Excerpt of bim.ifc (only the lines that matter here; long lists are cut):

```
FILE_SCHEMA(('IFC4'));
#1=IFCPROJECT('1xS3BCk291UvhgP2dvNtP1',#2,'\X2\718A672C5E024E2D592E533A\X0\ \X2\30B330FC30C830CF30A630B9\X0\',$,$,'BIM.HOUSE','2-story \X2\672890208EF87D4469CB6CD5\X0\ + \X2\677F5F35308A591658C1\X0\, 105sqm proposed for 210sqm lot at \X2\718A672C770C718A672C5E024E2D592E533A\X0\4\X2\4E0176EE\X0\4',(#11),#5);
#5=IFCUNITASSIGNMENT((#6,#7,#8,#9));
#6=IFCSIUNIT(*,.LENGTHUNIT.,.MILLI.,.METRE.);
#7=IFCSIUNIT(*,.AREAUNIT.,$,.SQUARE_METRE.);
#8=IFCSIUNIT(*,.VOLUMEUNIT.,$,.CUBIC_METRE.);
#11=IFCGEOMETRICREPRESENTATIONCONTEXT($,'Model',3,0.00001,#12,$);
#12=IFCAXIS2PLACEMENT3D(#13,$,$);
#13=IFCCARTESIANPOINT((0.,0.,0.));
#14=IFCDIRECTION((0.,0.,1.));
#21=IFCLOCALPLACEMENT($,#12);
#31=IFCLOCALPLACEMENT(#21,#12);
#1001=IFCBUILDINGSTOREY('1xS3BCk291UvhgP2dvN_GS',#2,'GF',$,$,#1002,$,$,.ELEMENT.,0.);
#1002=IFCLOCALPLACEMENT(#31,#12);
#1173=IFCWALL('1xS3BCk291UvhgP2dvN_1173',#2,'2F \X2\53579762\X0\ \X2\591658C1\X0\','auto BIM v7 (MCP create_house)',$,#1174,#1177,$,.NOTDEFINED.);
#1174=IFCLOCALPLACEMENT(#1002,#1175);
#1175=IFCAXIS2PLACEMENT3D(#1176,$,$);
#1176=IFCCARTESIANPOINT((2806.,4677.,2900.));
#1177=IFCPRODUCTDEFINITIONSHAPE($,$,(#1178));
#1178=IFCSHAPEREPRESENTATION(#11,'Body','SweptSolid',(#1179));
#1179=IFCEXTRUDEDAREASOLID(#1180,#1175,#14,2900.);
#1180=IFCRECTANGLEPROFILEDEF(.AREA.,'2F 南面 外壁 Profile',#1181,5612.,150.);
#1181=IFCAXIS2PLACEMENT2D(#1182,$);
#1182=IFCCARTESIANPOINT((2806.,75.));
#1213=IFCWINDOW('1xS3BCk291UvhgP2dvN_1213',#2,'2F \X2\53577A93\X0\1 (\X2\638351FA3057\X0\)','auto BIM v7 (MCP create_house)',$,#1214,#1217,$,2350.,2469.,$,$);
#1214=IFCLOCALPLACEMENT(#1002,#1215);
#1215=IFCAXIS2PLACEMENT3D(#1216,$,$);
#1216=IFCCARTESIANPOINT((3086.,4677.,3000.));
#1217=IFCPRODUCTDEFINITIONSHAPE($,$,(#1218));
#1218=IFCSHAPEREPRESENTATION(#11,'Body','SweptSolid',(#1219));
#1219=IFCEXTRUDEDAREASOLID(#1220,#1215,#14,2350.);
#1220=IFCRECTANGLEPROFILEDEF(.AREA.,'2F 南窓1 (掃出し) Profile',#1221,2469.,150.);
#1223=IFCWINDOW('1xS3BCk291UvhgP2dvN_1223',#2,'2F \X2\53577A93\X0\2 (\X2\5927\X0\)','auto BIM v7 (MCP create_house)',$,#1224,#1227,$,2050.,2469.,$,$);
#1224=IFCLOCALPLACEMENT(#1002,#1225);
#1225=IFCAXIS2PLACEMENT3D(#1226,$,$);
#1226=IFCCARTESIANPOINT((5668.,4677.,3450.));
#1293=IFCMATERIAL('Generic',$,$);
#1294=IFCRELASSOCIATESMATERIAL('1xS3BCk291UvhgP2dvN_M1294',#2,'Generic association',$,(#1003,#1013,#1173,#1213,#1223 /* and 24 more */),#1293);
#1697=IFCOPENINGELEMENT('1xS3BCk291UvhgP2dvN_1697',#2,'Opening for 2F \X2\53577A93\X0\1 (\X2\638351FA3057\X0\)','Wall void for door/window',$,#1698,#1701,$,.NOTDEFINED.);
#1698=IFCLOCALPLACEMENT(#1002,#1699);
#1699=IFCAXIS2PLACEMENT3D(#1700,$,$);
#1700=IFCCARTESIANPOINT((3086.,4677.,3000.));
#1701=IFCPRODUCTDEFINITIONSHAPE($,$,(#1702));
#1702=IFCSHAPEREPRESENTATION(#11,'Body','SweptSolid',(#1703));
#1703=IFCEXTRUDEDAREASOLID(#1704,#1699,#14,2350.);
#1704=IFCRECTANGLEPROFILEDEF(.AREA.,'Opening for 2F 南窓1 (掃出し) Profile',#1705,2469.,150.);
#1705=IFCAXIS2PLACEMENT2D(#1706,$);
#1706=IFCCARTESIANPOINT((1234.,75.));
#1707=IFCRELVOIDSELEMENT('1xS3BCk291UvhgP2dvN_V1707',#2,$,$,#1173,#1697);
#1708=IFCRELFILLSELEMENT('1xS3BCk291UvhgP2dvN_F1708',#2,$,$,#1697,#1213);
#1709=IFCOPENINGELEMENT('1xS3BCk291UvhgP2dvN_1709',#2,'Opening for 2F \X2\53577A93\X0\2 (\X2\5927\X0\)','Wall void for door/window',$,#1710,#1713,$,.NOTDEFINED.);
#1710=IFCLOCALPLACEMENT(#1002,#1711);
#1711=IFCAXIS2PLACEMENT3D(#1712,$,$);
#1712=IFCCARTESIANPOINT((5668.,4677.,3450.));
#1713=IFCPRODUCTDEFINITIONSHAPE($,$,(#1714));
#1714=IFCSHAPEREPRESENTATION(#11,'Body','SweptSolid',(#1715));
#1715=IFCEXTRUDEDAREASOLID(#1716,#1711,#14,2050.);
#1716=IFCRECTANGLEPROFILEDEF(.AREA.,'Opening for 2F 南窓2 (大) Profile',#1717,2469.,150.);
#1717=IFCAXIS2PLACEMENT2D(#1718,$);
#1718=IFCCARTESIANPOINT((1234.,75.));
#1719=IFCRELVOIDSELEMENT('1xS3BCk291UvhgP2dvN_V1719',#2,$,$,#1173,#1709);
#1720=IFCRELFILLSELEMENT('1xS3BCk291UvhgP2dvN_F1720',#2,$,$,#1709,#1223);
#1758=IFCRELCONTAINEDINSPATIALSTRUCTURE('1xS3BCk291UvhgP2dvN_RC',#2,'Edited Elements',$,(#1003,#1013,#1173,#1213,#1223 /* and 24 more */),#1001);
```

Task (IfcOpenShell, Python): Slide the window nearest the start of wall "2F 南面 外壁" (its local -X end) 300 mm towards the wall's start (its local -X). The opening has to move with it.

```python
import ifcopenshell
import ifcopenshell.api.geometry
import ifcopenshell.util.placement
import ifcopenshell.util.unit

model = ifcopenshell.open("bim.ifc")
unit_scale = ifcopenshell.util.unit.calculate_unit_scale(model)

window = model.by_id(1213)
opening = window.FillsVoids[0].RelatingOpeningElement
wall = opening.VoidsElements[0].RelatingBuildingElement

wall_matrix = ifcopenshell.util.placement.get_local_placement(wall.ObjectPlacement)
shift = wall_matrix[:3, 0] * -0.3 / unit_scale
before = ifcopenshell.util.placement.get_local_placement(window.ObjectPlacement)[:3, 3].copy()

# The window is not placed relative to its opening, so move both.
for product in (opening, window):
    matrix = ifcopenshell.util.placement.get_local_placement(product.ObjectPlacement)
    matrix[:3, 3] += shift
    ifcopenshell.api.geometry.edit_object_placement(model, product=product, matrix=matrix, is_si=False)

after = ifcopenshell.util.placement.get_local_placement(window.ObjectPlacement)[:3, 3]
print("window moved by", (after - before).round(3) + 0.0)

model.write("bim_edited.ifc")
```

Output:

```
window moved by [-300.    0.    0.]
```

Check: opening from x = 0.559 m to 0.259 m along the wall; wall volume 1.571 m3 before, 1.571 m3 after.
